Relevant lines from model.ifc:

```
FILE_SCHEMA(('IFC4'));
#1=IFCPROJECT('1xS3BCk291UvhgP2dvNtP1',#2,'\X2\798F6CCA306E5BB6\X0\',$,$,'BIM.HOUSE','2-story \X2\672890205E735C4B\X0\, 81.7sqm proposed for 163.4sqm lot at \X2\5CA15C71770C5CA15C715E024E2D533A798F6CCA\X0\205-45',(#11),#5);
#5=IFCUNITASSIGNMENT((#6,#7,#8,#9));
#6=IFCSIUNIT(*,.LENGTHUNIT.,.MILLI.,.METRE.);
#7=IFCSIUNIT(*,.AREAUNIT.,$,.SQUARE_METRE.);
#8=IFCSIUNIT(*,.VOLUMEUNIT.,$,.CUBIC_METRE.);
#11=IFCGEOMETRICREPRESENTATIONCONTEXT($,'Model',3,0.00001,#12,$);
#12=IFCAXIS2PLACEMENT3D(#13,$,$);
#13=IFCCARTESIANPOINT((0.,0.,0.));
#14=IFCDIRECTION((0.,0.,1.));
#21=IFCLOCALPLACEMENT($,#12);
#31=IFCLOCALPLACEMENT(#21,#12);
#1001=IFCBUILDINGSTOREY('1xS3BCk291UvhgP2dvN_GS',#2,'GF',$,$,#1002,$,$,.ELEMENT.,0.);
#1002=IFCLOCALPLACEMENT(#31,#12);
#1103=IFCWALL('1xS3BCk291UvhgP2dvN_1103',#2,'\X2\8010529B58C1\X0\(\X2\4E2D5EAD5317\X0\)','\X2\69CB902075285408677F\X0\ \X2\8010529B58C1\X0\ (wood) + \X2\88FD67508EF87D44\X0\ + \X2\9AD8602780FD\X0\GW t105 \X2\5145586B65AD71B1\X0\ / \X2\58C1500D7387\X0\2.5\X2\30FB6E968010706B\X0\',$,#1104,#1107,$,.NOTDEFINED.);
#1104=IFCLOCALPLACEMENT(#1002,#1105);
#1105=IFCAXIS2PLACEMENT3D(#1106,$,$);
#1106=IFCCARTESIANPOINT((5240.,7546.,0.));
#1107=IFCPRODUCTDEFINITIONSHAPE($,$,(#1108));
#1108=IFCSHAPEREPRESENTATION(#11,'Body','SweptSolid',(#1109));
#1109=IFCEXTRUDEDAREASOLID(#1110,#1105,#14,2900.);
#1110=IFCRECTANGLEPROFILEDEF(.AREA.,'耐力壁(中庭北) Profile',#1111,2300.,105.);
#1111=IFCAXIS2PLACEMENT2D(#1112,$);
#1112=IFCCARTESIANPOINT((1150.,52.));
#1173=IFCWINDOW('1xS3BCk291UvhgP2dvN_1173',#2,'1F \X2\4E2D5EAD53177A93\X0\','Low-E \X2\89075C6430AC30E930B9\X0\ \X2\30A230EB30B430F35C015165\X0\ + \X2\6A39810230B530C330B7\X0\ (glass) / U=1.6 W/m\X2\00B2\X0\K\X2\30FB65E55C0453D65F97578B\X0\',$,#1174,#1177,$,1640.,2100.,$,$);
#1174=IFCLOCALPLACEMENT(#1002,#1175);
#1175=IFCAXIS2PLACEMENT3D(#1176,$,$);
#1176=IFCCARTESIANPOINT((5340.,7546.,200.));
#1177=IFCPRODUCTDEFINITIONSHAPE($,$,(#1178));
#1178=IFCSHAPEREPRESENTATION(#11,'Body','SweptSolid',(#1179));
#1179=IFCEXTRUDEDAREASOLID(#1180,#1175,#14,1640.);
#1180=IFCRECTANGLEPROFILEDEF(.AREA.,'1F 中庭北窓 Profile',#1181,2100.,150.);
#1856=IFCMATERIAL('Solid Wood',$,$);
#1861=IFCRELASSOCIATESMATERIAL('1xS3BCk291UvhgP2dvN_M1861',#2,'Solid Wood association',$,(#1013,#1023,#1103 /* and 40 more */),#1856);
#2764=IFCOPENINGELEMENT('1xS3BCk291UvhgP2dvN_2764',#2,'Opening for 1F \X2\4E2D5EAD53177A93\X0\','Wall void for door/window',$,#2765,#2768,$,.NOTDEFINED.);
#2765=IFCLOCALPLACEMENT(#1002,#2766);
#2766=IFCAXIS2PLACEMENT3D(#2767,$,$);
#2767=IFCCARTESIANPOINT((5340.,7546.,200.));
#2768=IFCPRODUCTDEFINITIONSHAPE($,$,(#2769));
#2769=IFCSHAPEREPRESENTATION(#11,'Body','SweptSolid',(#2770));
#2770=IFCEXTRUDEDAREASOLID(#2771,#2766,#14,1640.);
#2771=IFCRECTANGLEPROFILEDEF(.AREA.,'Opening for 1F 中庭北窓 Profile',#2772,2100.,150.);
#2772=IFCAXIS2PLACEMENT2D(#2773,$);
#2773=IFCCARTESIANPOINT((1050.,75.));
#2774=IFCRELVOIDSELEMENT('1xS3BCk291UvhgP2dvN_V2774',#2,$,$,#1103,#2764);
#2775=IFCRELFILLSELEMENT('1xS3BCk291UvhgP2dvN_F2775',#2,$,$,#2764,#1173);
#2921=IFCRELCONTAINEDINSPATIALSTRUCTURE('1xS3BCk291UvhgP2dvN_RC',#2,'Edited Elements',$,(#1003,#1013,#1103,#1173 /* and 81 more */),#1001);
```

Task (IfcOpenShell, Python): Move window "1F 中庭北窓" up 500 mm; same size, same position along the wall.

```python
import numpy as np
import ifcopenshell
import ifcopenshell.api.geometry
import ifcopenshell.util.placement
import ifcopenshell.util.unit

model = ifcopenshell.open("model.ifc")
unit_scale = ifcopenshell.util.unit.calculate_unit_scale(model)

window = model.by_guid("1xS3BCk291UvhgP2dvN_1173")
opening = window.FillsVoids[0].RelatingOpeningElement
dz = 0.5 / unit_scale

shift = np.array([0.0, 0.0, dz])
# The window is not placed relative to its opening, so move both.
for product in (opening, window):
    matrix = ifcopenshell.util.placement.get_local_placement(product.ObjectPlacement)
    matrix[:3, 3] += shift
    ifcopenshell.api.geometry.edit_object_placement(model, product=product, matrix=matrix, is_si=False)

print(f"moved by {dz * unit_scale:+.3f} m")

model.write("model_edited.ifc")
```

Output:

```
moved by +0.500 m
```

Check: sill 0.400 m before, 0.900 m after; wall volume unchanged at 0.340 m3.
